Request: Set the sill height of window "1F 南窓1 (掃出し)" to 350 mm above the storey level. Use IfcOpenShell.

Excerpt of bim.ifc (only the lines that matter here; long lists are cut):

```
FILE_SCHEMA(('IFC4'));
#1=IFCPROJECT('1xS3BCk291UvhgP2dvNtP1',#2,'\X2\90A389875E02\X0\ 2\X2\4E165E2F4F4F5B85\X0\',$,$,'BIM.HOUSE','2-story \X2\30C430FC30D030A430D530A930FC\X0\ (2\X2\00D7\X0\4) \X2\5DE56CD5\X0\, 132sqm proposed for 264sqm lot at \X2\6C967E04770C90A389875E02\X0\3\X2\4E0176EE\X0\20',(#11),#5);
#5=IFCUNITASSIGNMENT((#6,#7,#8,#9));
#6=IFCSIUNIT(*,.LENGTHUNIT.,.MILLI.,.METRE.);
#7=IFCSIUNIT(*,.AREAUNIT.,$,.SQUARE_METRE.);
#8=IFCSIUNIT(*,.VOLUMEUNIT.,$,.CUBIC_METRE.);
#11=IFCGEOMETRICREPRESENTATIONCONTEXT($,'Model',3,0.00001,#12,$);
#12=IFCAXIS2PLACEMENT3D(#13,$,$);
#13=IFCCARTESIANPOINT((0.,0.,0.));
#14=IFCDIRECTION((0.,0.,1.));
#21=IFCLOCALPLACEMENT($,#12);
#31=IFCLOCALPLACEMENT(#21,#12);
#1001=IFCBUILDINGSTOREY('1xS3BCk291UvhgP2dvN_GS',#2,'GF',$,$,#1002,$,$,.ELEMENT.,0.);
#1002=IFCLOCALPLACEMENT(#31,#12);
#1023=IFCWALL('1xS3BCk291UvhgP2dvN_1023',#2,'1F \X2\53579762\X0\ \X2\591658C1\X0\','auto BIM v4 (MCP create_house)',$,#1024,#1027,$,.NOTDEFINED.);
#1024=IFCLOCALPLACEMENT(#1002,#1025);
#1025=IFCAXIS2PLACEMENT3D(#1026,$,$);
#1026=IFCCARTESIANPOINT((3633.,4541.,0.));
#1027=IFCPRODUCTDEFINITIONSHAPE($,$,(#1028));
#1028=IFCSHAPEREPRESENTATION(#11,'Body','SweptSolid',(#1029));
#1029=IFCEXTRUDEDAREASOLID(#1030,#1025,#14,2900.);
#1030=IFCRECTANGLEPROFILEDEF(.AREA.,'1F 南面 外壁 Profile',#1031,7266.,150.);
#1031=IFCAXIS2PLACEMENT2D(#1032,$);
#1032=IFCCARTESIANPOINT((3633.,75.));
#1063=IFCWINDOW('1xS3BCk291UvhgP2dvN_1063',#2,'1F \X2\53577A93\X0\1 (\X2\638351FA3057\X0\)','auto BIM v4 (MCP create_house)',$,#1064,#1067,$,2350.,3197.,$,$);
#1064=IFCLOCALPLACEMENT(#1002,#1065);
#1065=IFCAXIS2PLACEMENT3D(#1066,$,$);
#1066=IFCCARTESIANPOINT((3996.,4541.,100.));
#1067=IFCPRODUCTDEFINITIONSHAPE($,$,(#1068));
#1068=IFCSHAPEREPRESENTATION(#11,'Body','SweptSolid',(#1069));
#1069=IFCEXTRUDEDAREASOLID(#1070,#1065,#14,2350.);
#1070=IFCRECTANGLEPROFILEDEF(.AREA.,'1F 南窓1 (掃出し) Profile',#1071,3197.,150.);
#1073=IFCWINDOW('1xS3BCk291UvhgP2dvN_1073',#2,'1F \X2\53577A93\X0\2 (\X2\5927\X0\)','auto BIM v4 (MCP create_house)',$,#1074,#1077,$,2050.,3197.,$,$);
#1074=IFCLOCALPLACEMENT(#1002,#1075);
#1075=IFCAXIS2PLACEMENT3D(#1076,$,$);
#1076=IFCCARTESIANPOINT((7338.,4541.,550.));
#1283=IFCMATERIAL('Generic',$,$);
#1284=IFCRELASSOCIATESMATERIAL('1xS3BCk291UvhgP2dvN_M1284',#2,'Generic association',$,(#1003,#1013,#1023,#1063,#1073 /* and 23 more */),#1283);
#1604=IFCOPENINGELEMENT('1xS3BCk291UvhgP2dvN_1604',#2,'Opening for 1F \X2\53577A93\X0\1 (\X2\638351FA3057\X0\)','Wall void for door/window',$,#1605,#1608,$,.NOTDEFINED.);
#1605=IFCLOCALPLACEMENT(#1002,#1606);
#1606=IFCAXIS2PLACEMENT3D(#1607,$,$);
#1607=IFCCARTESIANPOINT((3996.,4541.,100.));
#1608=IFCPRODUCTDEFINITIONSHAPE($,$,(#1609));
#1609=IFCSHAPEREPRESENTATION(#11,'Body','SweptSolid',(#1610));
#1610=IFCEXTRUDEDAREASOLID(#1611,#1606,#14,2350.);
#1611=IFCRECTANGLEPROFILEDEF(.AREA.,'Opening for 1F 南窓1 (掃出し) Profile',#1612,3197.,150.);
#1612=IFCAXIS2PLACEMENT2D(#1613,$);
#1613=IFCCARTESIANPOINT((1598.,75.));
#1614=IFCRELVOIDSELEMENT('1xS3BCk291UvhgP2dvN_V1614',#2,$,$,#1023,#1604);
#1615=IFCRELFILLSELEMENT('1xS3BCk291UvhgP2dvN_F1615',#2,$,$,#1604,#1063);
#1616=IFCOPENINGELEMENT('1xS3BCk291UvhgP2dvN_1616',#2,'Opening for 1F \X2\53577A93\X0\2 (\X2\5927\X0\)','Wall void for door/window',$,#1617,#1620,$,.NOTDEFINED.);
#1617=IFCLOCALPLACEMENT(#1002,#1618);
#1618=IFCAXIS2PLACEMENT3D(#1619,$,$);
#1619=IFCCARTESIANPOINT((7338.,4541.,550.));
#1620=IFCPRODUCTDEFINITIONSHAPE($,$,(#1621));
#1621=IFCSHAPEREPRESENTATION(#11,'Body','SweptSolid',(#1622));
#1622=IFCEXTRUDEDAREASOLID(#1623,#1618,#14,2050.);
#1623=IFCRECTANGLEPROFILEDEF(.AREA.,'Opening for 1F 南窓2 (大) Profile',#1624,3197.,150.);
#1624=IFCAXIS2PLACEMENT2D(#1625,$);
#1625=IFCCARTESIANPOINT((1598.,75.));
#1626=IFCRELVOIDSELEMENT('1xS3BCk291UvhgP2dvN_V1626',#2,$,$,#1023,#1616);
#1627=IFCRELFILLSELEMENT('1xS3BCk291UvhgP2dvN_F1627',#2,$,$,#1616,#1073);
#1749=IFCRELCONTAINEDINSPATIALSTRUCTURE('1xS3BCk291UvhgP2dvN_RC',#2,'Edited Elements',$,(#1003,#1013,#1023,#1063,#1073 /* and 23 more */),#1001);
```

```python
import numpy as np
import ifcopenshell
import ifcopenshell.api.geometry
import ifcopenshell.geom
import ifcopenshell.util.element
import ifcopenshell.util.placement
import ifcopenshell.util.shape
import ifcopenshell.util.unit

model = ifcopenshell.open("bim.ifc")
unit_scale = ifcopenshell.util.unit.calculate_unit_scale(model)

window = model.by_guid("1xS3BCk291UvhgP2dvN_1063")
opening = window.FillsVoids[0].RelatingOpeningElement
storey = ifcopenshell.util.element.get_container(window, ifc_class="IfcBuildingStorey")
level = ifcopenshell.util.placement.get_local_placement(storey.ObjectPlacement)[2, 3]

# The opening's origin need not be at the sill, so measure its lowest point.
shape = ifcopenshell.geom.create_shape(ifcopenshell.geom.settings(), opening)
bottom = ifcopenshell.util.shape.get_shape_bottom_elevation(shape, shape.geometry) / unit_scale
dz = level + 0.35 / unit_scale - bottom

shift = np.array([0.0, 0.0, dz])
# The window is not placed relative to its opening, so move both.
for product in (opening, window):
    matrix = ifcopenshell.util.placement.get_local_placement(product.ObjectPlacement)
    matrix[:3, 3] += shift
    ifcopenshell.api.geometry.edit_object_placement(model, product=product, matrix=matrix, is_si=False)

print(f"moved by {dz * unit_scale:+.3f} m")

model.write("bim_updated.ifc")
```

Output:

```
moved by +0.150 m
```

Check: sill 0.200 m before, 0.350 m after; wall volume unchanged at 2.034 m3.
